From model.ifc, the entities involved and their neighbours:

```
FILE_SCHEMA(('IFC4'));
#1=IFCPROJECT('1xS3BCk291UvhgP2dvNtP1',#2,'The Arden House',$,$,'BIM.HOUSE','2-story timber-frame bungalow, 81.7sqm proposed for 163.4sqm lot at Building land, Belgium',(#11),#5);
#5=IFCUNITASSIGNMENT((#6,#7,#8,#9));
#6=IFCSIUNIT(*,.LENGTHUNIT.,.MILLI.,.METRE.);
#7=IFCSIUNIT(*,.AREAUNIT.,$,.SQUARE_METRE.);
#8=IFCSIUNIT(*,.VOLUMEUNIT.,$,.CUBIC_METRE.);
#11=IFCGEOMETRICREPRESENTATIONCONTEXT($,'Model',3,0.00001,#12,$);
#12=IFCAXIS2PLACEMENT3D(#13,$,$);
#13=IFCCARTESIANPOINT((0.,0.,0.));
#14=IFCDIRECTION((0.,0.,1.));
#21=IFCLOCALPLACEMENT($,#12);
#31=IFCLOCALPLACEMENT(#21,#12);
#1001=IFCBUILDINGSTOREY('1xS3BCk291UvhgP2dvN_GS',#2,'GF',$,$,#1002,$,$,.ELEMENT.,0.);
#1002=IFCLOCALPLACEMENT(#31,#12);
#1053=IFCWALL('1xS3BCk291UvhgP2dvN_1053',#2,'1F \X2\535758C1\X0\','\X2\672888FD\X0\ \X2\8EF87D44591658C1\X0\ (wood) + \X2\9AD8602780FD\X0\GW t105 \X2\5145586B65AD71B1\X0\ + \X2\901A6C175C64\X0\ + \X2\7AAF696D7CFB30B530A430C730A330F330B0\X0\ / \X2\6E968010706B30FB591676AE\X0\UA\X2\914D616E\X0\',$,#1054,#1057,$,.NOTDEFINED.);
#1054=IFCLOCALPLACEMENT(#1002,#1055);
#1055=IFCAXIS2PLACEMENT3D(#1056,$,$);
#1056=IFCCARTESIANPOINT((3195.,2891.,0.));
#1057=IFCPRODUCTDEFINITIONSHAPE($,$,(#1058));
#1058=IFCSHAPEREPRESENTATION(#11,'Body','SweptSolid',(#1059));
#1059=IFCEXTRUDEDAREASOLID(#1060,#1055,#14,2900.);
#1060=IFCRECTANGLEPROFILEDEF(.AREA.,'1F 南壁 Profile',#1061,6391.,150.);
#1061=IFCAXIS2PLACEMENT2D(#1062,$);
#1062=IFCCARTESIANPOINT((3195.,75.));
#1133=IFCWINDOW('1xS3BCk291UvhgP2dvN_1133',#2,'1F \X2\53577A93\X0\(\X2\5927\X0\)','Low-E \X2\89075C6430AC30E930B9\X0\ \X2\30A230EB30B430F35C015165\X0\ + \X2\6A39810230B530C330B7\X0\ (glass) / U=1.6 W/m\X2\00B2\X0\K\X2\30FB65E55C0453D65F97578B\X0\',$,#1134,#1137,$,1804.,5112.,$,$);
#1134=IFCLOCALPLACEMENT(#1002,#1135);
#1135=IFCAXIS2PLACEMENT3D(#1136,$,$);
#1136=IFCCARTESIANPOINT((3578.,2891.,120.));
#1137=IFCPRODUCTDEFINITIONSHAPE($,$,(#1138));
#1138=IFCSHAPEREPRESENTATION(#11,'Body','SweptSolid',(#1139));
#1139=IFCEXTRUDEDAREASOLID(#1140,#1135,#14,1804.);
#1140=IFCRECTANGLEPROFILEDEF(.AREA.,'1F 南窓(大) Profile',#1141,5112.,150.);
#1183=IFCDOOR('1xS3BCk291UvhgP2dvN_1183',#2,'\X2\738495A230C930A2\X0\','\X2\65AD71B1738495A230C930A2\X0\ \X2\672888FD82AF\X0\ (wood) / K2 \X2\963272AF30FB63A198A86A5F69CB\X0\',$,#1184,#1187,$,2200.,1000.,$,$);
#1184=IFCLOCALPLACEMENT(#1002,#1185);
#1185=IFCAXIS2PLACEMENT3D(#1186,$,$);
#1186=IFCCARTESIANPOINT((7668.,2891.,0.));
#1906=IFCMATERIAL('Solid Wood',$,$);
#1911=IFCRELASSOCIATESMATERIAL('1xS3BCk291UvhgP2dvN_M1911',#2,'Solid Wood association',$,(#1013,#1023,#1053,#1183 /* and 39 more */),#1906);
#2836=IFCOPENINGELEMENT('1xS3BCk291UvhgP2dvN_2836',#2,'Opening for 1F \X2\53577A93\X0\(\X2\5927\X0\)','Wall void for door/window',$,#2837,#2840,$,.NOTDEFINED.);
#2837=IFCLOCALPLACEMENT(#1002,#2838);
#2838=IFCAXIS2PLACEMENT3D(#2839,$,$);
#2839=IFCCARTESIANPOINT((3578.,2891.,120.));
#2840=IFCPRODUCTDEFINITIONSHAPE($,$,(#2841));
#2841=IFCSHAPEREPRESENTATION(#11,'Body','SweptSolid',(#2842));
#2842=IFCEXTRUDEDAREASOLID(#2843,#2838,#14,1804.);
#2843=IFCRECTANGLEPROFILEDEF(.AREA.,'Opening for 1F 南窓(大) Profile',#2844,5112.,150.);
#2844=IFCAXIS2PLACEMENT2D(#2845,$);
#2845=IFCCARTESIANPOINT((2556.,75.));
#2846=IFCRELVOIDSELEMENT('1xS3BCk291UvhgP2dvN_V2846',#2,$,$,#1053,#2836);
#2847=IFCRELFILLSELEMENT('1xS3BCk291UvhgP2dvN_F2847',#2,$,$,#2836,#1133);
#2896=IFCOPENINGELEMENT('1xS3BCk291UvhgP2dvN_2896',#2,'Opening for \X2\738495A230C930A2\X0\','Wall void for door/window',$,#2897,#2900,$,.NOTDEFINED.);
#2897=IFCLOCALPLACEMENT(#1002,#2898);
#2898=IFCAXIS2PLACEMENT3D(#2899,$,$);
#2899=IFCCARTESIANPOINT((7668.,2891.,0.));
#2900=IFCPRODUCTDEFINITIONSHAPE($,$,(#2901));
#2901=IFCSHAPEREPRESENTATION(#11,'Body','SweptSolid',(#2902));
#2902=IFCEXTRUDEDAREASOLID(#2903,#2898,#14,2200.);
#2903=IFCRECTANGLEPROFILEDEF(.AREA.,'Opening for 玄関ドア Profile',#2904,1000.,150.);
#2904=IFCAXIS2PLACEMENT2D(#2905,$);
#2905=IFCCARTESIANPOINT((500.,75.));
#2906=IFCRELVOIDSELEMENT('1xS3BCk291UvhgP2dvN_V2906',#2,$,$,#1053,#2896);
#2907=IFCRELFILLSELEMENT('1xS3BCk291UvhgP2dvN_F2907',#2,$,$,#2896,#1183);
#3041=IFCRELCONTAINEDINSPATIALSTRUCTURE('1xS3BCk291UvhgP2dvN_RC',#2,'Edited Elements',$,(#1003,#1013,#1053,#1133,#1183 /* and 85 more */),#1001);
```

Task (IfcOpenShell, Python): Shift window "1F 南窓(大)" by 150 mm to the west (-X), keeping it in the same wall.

```python
import ifcopenshell
import ifcopenshell.api.geometry
import ifcopenshell.util.placement
import ifcopenshell.util.unit

model = ifcopenshell.open("model.ifc")
unit_scale = ifcopenshell.util.unit.calculate_unit_scale(model)

window = model.by_id(1133)
opening = window.FillsVoids[0].RelatingOpeningElement
wall = opening.VoidsElements[0].RelatingBuildingElement

wall_matrix = ifcopenshell.util.placement.get_local_placement(wall.ObjectPlacement)
shift = wall_matrix[:3, 0] * -0.15 / unit_scale
before = ifcopenshell.util.placement.get_local_placement(window.ObjectPlacement)[:3, 3].copy()

# The window is not placed relative to its opening, so move both.
for product in (opening, window):
    matrix = ifcopenshell.util.placement.get_local_placement(product.ObjectPlacement)
    matrix[:3, 3] += shift
    ifcopenshell.api.geometry.edit_object_placement(model, product=product, matrix=matrix, is_si=False)

after = ifcopenshell.util.placement.get_local_placement(window.ObjectPlacement)[:3, 3]
print("window moved by", (after - before).round(3) + 0.0)

model.write("model-out.ifc")
```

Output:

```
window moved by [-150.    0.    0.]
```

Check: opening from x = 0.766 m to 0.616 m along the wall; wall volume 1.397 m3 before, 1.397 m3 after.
